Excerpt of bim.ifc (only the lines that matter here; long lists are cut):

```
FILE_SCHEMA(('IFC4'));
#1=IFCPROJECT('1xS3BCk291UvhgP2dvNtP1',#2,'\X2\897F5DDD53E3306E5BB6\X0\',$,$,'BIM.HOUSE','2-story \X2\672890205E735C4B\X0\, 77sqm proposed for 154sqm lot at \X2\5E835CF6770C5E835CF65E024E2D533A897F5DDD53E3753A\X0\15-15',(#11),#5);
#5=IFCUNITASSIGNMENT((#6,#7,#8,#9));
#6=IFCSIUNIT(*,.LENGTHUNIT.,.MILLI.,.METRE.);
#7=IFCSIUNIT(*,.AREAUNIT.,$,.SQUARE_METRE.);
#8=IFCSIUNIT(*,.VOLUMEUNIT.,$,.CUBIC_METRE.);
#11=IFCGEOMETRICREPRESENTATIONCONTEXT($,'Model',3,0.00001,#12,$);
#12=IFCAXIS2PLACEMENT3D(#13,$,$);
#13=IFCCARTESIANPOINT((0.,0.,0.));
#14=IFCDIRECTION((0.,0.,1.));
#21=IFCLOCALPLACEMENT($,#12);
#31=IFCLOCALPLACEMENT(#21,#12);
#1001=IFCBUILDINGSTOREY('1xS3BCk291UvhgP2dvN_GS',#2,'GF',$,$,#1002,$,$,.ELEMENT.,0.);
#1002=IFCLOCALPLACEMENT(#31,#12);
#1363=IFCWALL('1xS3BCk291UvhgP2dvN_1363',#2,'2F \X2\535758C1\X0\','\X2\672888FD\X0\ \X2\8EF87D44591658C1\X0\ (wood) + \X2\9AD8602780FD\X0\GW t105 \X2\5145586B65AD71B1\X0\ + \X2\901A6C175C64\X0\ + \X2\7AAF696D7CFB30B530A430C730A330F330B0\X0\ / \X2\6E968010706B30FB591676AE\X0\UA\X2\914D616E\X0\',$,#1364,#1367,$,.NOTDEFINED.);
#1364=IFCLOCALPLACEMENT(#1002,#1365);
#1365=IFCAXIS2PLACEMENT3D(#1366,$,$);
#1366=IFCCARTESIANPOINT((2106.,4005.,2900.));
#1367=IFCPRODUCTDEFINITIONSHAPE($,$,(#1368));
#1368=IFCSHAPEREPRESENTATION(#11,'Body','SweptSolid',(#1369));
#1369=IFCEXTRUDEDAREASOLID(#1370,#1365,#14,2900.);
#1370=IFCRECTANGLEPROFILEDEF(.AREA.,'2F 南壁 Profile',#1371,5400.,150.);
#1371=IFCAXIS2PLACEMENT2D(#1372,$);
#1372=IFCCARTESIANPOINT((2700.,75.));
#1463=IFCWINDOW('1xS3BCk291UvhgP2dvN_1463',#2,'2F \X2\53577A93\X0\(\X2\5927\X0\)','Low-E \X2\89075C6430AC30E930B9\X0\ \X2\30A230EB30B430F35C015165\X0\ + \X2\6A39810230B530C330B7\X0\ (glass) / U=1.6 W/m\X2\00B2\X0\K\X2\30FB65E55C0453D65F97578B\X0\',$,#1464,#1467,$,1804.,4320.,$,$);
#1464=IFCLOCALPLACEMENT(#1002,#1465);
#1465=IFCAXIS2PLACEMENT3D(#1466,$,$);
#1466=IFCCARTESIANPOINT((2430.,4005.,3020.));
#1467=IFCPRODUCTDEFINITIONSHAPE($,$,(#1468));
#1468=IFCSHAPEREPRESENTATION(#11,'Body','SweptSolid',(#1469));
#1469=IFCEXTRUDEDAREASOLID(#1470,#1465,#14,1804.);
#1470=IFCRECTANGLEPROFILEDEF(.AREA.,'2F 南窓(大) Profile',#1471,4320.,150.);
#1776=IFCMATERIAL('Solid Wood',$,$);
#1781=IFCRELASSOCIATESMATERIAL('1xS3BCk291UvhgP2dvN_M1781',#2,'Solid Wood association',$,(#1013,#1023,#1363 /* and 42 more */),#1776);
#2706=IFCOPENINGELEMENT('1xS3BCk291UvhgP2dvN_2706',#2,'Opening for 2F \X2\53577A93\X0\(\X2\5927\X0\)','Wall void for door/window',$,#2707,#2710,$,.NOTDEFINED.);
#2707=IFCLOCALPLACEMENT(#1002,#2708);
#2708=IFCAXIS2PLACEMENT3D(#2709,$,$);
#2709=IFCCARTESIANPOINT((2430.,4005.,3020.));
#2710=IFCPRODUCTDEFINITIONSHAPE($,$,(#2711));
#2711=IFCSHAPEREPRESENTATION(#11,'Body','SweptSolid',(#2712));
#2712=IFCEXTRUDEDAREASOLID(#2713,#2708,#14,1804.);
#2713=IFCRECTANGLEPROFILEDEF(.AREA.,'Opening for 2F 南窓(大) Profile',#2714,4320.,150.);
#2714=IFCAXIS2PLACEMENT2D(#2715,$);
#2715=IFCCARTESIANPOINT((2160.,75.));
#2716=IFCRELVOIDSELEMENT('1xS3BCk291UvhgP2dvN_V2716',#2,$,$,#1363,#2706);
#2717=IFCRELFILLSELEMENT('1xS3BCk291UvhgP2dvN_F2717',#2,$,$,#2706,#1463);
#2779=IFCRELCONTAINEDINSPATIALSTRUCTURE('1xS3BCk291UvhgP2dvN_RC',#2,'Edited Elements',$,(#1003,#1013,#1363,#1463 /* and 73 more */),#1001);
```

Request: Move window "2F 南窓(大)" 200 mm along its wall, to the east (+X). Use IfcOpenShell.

```python
import ifcopenshell
import ifcopenshell.api.geometry
import ifcopenshell.util.placement
import ifcopenshell.util.unit

model = ifcopenshell.open("bim.ifc")
unit_scale = ifcopenshell.util.unit.calculate_unit_scale(model)

window = model.by_guid("1xS3BCk291UvhgP2dvN_1463")
opening = window.FillsVoids[0].RelatingOpeningElement
wall = opening.VoidsElements[0].RelatingBuildingElement

wall_matrix = ifcopenshell.util.placement.get_local_placement(wall.ObjectPlacement)
shift = wall_matrix[:3, 0] * 0.2 / unit_scale
before = ifcopenshell.util.placement.get_local_placement(window.ObjectPlacement)[:3, 3].copy()

# The window is not placed relative to its opening, so move both.
for product in (opening, window):
    matrix = ifcopenshell.util.placement.get_local_placement(product.ObjectPlacement)
    matrix[:3, 3] += shift
    ifcopenshell.api.geometry.edit_object_placement(model, product=product, matrix=matrix, is_si=False)

after = ifcopenshell.util.placement.get_local_placement(window.ObjectPlacement)[:3, 3]
print("window moved by", (after - before).round(3) + 0.0)

model.write("bim-out.ifc")
```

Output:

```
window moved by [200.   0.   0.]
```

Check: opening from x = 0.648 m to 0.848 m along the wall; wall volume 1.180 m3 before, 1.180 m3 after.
